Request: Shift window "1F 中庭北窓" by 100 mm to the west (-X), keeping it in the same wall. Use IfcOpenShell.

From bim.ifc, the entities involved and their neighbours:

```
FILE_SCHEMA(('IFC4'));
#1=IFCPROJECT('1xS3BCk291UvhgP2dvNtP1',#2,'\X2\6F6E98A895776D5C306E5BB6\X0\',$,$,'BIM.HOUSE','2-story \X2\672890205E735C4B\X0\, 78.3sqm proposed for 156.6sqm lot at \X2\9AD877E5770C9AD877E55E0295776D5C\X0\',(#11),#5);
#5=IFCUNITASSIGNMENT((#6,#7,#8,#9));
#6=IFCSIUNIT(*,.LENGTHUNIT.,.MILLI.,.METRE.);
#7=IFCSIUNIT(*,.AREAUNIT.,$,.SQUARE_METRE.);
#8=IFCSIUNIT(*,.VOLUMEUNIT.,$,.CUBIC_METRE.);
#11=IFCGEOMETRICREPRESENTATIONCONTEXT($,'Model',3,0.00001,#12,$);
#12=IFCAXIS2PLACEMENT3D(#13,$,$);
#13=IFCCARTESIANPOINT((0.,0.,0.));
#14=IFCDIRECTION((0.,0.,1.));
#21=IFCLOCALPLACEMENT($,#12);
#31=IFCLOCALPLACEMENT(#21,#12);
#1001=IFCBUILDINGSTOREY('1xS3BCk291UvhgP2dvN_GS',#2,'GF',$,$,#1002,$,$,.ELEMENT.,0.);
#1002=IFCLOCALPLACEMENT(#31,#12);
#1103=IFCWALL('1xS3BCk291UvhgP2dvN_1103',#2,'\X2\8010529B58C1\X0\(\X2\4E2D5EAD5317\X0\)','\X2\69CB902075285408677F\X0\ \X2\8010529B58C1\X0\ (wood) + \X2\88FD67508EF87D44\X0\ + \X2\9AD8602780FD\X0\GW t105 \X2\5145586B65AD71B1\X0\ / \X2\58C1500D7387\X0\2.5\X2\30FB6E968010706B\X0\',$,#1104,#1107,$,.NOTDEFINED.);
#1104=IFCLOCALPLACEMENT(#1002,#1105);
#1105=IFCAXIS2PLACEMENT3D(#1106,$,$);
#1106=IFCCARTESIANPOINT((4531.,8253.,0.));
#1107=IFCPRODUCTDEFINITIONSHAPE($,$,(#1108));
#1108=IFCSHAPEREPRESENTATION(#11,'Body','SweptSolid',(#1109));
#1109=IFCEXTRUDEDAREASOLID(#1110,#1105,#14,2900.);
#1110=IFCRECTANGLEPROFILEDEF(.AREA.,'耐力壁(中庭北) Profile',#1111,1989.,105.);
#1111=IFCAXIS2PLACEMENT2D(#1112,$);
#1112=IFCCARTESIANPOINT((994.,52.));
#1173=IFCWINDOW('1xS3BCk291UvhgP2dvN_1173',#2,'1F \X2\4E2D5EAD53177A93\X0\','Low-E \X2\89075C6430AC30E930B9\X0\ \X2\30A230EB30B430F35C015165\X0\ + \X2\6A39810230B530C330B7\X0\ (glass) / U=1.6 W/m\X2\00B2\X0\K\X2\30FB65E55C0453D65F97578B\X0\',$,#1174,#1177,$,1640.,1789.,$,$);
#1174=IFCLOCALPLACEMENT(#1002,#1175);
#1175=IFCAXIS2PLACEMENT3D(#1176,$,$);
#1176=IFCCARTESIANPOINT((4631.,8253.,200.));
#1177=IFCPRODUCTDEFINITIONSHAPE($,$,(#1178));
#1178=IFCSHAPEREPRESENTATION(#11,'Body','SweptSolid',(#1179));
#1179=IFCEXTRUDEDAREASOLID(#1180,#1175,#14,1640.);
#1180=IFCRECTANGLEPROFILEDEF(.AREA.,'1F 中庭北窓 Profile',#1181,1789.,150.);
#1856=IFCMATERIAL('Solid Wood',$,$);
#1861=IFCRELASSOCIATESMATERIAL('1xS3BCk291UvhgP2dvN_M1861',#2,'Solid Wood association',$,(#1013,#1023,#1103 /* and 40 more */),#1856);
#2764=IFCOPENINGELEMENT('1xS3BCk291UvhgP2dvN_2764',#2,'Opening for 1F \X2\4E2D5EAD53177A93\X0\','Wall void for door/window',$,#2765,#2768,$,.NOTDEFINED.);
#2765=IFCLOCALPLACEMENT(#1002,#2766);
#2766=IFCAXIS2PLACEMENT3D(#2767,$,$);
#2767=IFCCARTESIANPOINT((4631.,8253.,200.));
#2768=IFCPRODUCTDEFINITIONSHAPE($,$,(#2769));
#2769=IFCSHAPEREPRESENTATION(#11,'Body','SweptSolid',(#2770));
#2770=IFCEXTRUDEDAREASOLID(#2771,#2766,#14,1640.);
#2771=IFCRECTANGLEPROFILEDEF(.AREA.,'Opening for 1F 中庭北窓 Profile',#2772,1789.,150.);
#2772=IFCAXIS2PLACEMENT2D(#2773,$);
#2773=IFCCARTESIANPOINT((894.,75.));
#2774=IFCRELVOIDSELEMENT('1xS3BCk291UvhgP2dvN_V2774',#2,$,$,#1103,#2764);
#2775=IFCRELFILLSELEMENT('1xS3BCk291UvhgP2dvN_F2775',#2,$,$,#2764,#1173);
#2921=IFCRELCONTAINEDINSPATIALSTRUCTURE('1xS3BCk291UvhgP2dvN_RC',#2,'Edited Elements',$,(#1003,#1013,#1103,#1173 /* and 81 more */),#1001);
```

```python
import ifcopenshell
import ifcopenshell.api.geometry
import ifcopenshell.util.placement
import ifcopenshell.util.unit

model = ifcopenshell.open("bim.ifc")
unit_scale = ifcopenshell.util.unit.calculate_unit_scale(model)

window = model.by_guid("1xS3BCk291UvhgP2dvN_1173")
opening = window.FillsVoids[0].RelatingOpeningElement
wall = opening.VoidsElements[0].RelatingBuildingElement

wall_matrix = ifcopenshell.util.placement.get_local_placement(wall.ObjectPlacement)
shift = wall_matrix[:3, 0] * -0.1 / unit_scale
before = ifcopenshell.util.placement.get_local_placement(window.ObjectPlacement)[:3, 3].copy()

# The window is not placed relative to its opening, so move both.
for product in (opening, window):
    matrix = ifcopenshell.util.placement.get_local_placement(product.ObjectPlacement)
    matrix[:3, 3] += shift
    ifcopenshell.api.geometry.edit_object_placement(model, product=product, matrix=matrix, is_si=False)

after = ifcopenshell.util.placement.get_local_placement(window.ObjectPlacement)[:3, 3]
print("window moved by", (after - before).round(3) + 0.0)

model.write("bim_v2.ifc")
```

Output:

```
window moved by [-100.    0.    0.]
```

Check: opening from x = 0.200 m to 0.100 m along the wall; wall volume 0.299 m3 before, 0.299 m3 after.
